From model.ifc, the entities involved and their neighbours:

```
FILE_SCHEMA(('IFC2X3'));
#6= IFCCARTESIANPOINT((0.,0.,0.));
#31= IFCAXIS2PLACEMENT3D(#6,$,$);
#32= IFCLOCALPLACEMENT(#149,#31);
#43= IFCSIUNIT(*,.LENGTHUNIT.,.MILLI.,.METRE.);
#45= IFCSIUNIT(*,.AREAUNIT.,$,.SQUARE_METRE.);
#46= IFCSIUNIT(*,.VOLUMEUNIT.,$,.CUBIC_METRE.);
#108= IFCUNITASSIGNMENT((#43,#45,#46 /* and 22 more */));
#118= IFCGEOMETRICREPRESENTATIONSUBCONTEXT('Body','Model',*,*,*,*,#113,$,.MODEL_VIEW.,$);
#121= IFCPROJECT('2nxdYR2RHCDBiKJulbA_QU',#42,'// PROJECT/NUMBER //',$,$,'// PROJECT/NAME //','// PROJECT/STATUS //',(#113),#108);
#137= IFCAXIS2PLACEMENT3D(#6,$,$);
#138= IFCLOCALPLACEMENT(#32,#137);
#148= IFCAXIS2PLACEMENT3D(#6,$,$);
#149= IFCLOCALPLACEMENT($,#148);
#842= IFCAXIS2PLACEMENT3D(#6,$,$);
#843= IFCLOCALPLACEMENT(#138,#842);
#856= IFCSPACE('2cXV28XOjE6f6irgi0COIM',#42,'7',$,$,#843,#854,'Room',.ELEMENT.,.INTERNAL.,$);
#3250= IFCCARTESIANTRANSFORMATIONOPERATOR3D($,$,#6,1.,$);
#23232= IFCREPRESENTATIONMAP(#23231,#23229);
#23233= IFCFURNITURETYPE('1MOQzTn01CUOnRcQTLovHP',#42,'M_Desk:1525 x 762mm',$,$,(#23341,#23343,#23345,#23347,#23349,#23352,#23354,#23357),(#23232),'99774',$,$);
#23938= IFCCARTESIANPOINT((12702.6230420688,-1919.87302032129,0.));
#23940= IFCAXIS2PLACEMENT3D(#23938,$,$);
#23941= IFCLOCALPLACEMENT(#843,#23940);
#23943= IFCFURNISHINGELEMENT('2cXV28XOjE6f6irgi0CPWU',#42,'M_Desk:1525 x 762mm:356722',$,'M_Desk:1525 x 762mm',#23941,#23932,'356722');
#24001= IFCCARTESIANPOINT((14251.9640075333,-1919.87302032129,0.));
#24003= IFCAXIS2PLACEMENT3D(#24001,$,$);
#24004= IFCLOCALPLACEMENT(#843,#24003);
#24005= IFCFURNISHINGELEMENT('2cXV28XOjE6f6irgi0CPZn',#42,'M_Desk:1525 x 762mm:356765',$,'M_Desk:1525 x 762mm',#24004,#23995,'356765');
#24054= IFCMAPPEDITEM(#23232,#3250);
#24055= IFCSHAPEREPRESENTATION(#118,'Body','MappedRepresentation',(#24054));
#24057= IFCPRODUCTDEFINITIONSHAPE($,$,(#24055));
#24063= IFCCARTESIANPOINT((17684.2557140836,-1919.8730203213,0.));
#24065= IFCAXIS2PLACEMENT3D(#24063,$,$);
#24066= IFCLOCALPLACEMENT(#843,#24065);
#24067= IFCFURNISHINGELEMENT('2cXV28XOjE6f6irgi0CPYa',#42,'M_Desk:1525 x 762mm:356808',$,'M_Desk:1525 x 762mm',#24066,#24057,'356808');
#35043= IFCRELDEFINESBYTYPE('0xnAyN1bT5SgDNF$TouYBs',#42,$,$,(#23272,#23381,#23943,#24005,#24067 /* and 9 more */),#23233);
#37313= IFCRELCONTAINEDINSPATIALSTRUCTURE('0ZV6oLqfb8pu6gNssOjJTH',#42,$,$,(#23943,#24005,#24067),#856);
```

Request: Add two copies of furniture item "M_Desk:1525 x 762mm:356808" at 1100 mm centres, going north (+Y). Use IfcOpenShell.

```python
import numpy as np
import ifcopenshell
import ifcopenshell.api.geometry
import ifcopenshell.api.root
import ifcopenshell.util.element
import ifcopenshell.util.placement
import ifcopenshell.util.unit

model = ifcopenshell.open("model.ifc")
unit_scale = ifcopenshell.util.unit.calculate_unit_scale(model)


def reuse_history(source, copy):
    """copy_class also copies each property set's owner history, people and application; keep the originals."""
    for rel in copy.IsDefinedBy:
        if rel.is_a("IfcRelDefinesByProperties") and (history := rel.RelatingPropertyDefinition.OwnerHistory):
            rel.RelatingPropertyDefinition.OwnerHistory = source.OwnerHistory
            ifcopenshell.util.element.remove_deep2(model, history)


source = model.by_id(24067)
base = ifcopenshell.util.placement.get_local_placement(source.ObjectPlacement)
step = np.array([0.0, 1.0, 0.0]) * 1.1 / unit_scale

for i in range(1, 3):
    copy = ifcopenshell.api.root.copy_class(model, product=source)
    copy.Representation = ifcopenshell.util.element.copy_deep(
        model, source.Representation, exclude=["IfcGeometricRepresentationContext", "IfcRepresentationMap"]
    )
    copy.Name = "M_Desk:1525 x 762mm"
    copy.Tag = None
    reuse_history(source, copy)
    matrix = base.copy()
    matrix[:3, 3] += i * step
    print("added at", matrix[:3, 3].round(3) + 0.0)
    ifcopenshell.api.geometry.edit_object_placement(model, product=copy, matrix=matrix, is_si=False)

model.write("model_v2.ifc")
```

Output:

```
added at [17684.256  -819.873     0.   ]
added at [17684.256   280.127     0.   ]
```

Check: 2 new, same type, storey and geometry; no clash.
